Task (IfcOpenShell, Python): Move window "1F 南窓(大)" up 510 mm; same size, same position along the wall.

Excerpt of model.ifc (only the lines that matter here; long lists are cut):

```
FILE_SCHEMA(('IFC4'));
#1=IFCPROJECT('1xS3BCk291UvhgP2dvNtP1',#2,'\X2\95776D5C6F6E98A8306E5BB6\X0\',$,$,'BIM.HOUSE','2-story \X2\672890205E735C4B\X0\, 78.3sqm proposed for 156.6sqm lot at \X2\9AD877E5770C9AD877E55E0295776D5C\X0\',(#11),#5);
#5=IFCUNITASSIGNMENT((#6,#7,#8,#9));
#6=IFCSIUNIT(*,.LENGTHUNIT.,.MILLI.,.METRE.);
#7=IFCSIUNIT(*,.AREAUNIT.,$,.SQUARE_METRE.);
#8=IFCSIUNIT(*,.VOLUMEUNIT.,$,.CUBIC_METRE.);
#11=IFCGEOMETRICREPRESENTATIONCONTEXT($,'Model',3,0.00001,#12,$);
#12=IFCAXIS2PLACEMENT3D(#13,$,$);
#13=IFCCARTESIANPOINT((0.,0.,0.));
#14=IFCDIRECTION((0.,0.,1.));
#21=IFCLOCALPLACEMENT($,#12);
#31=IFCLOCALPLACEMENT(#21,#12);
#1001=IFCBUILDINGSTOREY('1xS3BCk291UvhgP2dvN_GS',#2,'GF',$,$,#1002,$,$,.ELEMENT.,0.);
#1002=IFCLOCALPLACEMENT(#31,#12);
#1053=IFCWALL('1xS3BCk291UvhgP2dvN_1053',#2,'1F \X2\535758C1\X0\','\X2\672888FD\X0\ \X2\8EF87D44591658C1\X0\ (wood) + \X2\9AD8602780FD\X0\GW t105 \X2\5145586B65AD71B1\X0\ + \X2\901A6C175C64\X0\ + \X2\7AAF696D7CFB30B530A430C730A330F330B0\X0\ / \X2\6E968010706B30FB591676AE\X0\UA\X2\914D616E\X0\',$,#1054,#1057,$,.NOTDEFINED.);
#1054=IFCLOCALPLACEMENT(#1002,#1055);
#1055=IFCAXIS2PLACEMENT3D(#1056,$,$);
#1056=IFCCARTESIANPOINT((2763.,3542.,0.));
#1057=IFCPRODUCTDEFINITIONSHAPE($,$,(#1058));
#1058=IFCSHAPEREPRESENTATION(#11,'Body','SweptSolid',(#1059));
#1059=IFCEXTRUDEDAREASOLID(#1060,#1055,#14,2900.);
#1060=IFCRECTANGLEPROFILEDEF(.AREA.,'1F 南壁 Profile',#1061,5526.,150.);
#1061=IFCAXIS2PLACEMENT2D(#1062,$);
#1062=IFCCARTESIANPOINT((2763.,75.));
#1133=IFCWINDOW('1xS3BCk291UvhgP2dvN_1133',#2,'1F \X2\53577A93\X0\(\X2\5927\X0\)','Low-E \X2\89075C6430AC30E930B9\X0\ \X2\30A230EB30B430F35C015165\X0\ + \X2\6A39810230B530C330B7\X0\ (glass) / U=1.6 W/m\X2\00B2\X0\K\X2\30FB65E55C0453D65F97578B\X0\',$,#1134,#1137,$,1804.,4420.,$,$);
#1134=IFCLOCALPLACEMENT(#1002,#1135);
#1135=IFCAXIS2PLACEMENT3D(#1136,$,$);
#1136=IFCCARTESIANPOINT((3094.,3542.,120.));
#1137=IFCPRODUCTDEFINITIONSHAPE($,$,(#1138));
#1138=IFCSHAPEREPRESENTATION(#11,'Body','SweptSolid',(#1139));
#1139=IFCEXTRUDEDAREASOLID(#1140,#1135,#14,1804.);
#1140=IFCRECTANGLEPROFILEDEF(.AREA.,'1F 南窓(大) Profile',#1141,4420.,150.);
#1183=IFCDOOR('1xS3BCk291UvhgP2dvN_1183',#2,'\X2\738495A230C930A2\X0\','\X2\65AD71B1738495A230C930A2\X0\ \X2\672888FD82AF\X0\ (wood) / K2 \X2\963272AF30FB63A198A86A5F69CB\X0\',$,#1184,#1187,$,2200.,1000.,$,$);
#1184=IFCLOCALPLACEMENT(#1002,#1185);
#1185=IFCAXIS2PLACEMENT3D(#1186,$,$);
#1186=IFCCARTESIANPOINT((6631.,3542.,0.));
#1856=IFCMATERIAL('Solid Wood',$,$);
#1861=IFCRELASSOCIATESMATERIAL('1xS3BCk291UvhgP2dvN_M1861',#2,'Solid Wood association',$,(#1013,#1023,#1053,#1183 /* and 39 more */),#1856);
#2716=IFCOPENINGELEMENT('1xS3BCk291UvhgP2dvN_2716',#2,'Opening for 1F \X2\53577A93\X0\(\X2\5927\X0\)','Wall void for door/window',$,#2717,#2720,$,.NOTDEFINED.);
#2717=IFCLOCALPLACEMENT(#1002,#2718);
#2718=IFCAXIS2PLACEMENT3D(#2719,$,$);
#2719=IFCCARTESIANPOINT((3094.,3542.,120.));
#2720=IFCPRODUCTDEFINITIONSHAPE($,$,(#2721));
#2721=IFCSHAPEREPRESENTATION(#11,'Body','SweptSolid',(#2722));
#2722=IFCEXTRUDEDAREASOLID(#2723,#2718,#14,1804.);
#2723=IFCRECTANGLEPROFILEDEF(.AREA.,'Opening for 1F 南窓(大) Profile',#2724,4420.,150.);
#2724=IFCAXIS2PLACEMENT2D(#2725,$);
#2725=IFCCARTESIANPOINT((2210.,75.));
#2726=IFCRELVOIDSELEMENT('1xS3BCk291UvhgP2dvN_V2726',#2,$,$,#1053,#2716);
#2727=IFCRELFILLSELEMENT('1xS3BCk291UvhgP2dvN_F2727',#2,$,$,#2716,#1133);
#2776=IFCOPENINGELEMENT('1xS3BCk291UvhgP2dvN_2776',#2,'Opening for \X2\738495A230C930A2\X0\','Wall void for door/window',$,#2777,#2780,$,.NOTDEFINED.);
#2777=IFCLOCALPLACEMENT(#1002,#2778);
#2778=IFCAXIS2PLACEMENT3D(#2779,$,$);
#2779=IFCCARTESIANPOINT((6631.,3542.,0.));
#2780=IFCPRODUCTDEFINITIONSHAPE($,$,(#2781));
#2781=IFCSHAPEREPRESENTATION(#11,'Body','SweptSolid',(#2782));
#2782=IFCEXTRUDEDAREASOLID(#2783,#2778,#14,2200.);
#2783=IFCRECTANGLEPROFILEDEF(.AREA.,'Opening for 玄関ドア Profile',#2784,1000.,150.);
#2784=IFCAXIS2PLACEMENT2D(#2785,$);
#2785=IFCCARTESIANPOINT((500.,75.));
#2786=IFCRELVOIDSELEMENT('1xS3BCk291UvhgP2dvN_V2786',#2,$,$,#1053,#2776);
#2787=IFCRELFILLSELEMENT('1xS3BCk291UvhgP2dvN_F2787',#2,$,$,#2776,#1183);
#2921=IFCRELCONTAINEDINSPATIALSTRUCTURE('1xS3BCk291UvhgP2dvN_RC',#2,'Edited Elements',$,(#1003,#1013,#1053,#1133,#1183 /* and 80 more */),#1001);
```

```python
import numpy as np
import ifcopenshell
import ifcopenshell.api.geometry
import ifcopenshell.util.placement
import ifcopenshell.util.unit

model = ifcopenshell.open("model.ifc")
unit_scale = ifcopenshell.util.unit.calculate_unit_scale(model)

window = model.by_guid("1xS3BCk291UvhgP2dvN_1133")
opening = window.FillsVoids[0].RelatingOpeningElement
dz = 510.0

shift = np.array([0.0, 0.0, dz])
# The window is not placed relative to its opening, so move both.
for product in (opening, window):
    matrix = ifcopenshell.util.placement.get_local_placement(product.ObjectPlacement)
    matrix[:3, 3] += shift
    ifcopenshell.api.geometry.edit_object_placement(model, product=product, matrix=matrix, is_si=False)

print(f"moved by {dz * unit_scale:+.3f} m")

model.write("model_rev.ifc")
```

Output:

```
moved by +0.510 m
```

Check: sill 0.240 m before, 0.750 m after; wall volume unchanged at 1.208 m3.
